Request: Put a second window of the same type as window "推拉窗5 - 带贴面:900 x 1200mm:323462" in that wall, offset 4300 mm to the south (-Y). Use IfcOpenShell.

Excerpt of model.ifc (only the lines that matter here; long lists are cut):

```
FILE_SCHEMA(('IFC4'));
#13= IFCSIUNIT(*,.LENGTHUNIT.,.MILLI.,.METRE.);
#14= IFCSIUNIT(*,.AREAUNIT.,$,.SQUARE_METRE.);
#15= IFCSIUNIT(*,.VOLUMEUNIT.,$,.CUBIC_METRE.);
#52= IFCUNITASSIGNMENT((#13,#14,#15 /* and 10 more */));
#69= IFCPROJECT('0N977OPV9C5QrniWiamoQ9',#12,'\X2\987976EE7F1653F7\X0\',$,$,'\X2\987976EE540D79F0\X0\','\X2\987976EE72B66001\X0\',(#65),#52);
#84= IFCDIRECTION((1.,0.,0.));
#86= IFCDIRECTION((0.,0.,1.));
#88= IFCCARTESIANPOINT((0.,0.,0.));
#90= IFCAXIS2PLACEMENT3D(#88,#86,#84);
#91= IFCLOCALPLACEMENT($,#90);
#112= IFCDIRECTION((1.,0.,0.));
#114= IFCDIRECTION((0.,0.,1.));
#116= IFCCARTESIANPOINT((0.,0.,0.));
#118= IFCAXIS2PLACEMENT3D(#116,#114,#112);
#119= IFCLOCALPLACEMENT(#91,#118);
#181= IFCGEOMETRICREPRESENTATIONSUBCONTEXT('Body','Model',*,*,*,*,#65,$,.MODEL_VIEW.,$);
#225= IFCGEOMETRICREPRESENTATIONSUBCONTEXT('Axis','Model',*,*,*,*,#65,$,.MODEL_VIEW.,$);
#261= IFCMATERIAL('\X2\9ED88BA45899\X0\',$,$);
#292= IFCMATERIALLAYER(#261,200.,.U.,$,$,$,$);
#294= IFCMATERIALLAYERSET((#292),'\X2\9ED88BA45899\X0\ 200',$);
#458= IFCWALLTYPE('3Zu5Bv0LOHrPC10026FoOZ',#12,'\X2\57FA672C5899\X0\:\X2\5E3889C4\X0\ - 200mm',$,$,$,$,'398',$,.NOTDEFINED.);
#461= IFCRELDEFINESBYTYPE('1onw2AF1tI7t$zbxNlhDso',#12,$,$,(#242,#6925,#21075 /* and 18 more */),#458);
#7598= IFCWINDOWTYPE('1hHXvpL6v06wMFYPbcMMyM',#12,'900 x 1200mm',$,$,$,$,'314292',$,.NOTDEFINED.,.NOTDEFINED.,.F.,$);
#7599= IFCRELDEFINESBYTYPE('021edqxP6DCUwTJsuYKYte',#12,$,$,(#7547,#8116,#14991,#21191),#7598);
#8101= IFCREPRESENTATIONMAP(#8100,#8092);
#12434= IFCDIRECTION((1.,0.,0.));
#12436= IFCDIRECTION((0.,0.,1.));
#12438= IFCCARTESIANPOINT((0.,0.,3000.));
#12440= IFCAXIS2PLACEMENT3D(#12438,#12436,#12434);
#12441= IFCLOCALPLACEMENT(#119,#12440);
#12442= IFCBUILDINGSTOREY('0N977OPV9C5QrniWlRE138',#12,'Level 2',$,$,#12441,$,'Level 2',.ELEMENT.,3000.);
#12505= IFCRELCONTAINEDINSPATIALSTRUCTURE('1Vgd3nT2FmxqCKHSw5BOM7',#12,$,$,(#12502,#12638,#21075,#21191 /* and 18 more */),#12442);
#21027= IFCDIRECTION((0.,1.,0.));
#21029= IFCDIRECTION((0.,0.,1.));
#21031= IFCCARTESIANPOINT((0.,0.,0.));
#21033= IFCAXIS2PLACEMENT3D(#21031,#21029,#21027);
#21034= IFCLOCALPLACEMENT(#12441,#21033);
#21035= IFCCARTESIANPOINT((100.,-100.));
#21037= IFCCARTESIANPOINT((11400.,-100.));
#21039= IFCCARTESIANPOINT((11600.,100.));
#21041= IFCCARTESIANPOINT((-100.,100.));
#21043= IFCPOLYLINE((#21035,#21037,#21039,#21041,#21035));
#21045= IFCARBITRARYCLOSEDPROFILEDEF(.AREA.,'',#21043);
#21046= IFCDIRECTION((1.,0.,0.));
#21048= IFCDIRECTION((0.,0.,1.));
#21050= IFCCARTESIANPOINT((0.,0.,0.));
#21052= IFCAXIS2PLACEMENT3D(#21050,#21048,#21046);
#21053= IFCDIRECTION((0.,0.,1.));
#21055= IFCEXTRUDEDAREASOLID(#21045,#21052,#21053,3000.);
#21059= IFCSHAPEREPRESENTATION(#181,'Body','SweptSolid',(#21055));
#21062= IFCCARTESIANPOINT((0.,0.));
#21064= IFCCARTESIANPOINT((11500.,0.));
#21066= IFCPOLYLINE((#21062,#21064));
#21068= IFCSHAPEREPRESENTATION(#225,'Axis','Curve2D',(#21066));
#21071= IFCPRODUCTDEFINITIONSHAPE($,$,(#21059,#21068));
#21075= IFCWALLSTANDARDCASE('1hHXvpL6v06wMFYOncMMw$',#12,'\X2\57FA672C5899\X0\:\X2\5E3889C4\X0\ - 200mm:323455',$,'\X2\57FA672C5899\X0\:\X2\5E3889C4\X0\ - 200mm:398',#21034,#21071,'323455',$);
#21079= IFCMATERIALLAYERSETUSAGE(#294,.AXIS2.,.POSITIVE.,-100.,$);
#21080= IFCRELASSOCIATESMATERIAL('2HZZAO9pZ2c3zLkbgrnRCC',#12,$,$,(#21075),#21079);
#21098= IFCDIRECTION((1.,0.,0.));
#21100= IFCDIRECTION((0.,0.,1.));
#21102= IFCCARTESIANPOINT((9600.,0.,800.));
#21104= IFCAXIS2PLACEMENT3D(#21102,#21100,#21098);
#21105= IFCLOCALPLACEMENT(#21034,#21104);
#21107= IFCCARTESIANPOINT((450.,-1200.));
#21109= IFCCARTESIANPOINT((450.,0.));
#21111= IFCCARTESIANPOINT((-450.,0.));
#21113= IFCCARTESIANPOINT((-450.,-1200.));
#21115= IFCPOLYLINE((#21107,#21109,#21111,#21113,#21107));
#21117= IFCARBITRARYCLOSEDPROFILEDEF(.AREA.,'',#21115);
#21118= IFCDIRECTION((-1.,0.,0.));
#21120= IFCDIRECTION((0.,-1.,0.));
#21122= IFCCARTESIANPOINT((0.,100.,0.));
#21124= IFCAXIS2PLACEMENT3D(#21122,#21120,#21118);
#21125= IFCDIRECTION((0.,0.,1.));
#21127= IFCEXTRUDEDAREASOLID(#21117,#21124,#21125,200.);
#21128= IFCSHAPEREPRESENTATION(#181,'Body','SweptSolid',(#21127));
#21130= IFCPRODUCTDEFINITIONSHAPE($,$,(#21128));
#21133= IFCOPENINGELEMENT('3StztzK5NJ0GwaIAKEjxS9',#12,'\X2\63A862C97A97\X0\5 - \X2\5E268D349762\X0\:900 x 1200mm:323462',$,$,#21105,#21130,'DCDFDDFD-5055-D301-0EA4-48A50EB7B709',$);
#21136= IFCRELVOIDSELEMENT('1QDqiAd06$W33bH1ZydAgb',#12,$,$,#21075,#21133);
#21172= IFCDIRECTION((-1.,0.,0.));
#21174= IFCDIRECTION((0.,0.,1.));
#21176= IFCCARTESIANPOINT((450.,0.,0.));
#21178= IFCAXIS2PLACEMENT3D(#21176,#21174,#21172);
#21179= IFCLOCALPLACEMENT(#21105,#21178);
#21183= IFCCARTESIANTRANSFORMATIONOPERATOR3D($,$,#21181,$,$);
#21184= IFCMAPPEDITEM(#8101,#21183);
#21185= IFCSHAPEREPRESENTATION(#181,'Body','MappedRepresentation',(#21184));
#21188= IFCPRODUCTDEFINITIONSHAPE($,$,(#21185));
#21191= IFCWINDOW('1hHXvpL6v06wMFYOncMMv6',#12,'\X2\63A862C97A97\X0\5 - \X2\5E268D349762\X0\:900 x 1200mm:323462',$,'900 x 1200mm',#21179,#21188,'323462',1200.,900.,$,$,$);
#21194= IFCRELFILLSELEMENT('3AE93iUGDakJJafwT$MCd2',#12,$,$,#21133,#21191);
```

```python
import ifcopenshell
import ifcopenshell.api.feature
import ifcopenshell.api.geometry
import ifcopenshell.api.root
import ifcopenshell.geom
import ifcopenshell.util.element
import ifcopenshell.util.placement
import ifcopenshell.util.shape

model = ifcopenshell.open("model.ifc")
settings = ifcopenshell.geom.settings()


def volume(element):
    """Net volume in cubic metres, openings subtracted."""
    shape = ifcopenshell.geom.create_shape(settings, element)
    return ifcopenshell.util.shape.get_volume(shape.geometry)


def reuse_history(source, copy):
    """copy_class also copies each property set's owner history, people and application; keep the originals."""
    for rel in copy.IsDefinedBy:
        if rel.is_a("IfcRelDefinesByProperties") and (history := rel.RelatingPropertyDefinition.OwnerHistory):
            rel.RelatingPropertyDefinition.OwnerHistory = source.OwnerHistory
            ifcopenshell.util.element.remove_deep2(model, history)


window = model.by_guid("1hHXvpL6v06wMFYOncMMv6")
opening = window.FillsVoids[0].RelatingOpeningElement
wall = opening.VoidsElements[0].RelatingBuildingElement
before = volume(wall)
shift = ifcopenshell.util.placement.get_local_placement(wall.ObjectPlacement)[:3, 0] * -4300.0

# copy_class copies the void relationship, type, container and properties, but no geometry.
new_opening = ifcopenshell.api.root.copy_class(model, product=opening)
new_opening.Representation = ifcopenshell.util.element.copy_deep(
    model, opening.Representation, exclude=["IfcGeometricRepresentationContext", "IfcRepresentationMap"]
)
new_opening.Name = "推拉窗5 - 带贴面:900 x 1200mm"
new_opening.Tag = None
new_window = ifcopenshell.api.root.copy_class(model, product=window)
new_window.Representation = ifcopenshell.util.element.copy_deep(
    model, window.Representation, exclude=["IfcGeometricRepresentationContext", "IfcRepresentationMap"]
)
new_window.Name = "推拉窗5 - 带贴面:900 x 1200mm"
new_window.Tag = None
reuse_history(window, new_window)
ifcopenshell.api.feature.add_filling(model, opening=new_opening, element=new_window)

for old, new in ((opening, new_opening), (window, new_window)):
    matrix = ifcopenshell.util.placement.get_local_placement(old.ObjectPlacement)
    matrix[:3, 3] += shift
    ifcopenshell.api.geometry.edit_object_placement(model, product=new, matrix=matrix, is_si=False)

after = volume(wall)

print(f"wall volume {before:.3f} -> {after:.3f} m3")

model.write("model_updated.ifc")
```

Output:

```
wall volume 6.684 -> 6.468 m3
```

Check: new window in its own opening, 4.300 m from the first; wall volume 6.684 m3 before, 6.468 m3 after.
